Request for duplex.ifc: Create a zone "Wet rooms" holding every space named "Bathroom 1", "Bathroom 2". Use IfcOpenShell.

First a look at what the model holds.

```python
import ifcopenshell

model = ifcopenshell.open("duplex.ifc")
print(model.schema)
seen = {}
for space in model.by_type("IfcSpace"):
    seen[space.LongName] = seen.get(space.LongName, 0) + 1
for name, count in sorted(seen.items(), key=str):
    print(count, "x", name)
print("zones:", [z.Name for z in model.by_type("IfcZone")][:20])
```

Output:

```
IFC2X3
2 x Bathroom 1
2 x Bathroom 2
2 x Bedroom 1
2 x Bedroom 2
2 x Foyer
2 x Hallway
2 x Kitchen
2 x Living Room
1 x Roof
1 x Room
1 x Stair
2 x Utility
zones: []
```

```python
import ifcopenshell
import ifcopenshell.api.group
import ifcopenshell.api.root

model = ifcopenshell.open("duplex.ifc")

names = {"Bathroom 1", "Bathroom 2"}
spaces = [s for s in model.by_type("IfcSpace") if s.LongName in names]

zone = ifcopenshell.api.root.create_entity(model, ifc_class="IfcZone", name="Wet rooms")
ifcopenshell.api.group.assign_group(model, products=spaces, group=zone)
print(len(spaces), "spaces in", zone.Name)

model.write("duplex_v2.ifc")
```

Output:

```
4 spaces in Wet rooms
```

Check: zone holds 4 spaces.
